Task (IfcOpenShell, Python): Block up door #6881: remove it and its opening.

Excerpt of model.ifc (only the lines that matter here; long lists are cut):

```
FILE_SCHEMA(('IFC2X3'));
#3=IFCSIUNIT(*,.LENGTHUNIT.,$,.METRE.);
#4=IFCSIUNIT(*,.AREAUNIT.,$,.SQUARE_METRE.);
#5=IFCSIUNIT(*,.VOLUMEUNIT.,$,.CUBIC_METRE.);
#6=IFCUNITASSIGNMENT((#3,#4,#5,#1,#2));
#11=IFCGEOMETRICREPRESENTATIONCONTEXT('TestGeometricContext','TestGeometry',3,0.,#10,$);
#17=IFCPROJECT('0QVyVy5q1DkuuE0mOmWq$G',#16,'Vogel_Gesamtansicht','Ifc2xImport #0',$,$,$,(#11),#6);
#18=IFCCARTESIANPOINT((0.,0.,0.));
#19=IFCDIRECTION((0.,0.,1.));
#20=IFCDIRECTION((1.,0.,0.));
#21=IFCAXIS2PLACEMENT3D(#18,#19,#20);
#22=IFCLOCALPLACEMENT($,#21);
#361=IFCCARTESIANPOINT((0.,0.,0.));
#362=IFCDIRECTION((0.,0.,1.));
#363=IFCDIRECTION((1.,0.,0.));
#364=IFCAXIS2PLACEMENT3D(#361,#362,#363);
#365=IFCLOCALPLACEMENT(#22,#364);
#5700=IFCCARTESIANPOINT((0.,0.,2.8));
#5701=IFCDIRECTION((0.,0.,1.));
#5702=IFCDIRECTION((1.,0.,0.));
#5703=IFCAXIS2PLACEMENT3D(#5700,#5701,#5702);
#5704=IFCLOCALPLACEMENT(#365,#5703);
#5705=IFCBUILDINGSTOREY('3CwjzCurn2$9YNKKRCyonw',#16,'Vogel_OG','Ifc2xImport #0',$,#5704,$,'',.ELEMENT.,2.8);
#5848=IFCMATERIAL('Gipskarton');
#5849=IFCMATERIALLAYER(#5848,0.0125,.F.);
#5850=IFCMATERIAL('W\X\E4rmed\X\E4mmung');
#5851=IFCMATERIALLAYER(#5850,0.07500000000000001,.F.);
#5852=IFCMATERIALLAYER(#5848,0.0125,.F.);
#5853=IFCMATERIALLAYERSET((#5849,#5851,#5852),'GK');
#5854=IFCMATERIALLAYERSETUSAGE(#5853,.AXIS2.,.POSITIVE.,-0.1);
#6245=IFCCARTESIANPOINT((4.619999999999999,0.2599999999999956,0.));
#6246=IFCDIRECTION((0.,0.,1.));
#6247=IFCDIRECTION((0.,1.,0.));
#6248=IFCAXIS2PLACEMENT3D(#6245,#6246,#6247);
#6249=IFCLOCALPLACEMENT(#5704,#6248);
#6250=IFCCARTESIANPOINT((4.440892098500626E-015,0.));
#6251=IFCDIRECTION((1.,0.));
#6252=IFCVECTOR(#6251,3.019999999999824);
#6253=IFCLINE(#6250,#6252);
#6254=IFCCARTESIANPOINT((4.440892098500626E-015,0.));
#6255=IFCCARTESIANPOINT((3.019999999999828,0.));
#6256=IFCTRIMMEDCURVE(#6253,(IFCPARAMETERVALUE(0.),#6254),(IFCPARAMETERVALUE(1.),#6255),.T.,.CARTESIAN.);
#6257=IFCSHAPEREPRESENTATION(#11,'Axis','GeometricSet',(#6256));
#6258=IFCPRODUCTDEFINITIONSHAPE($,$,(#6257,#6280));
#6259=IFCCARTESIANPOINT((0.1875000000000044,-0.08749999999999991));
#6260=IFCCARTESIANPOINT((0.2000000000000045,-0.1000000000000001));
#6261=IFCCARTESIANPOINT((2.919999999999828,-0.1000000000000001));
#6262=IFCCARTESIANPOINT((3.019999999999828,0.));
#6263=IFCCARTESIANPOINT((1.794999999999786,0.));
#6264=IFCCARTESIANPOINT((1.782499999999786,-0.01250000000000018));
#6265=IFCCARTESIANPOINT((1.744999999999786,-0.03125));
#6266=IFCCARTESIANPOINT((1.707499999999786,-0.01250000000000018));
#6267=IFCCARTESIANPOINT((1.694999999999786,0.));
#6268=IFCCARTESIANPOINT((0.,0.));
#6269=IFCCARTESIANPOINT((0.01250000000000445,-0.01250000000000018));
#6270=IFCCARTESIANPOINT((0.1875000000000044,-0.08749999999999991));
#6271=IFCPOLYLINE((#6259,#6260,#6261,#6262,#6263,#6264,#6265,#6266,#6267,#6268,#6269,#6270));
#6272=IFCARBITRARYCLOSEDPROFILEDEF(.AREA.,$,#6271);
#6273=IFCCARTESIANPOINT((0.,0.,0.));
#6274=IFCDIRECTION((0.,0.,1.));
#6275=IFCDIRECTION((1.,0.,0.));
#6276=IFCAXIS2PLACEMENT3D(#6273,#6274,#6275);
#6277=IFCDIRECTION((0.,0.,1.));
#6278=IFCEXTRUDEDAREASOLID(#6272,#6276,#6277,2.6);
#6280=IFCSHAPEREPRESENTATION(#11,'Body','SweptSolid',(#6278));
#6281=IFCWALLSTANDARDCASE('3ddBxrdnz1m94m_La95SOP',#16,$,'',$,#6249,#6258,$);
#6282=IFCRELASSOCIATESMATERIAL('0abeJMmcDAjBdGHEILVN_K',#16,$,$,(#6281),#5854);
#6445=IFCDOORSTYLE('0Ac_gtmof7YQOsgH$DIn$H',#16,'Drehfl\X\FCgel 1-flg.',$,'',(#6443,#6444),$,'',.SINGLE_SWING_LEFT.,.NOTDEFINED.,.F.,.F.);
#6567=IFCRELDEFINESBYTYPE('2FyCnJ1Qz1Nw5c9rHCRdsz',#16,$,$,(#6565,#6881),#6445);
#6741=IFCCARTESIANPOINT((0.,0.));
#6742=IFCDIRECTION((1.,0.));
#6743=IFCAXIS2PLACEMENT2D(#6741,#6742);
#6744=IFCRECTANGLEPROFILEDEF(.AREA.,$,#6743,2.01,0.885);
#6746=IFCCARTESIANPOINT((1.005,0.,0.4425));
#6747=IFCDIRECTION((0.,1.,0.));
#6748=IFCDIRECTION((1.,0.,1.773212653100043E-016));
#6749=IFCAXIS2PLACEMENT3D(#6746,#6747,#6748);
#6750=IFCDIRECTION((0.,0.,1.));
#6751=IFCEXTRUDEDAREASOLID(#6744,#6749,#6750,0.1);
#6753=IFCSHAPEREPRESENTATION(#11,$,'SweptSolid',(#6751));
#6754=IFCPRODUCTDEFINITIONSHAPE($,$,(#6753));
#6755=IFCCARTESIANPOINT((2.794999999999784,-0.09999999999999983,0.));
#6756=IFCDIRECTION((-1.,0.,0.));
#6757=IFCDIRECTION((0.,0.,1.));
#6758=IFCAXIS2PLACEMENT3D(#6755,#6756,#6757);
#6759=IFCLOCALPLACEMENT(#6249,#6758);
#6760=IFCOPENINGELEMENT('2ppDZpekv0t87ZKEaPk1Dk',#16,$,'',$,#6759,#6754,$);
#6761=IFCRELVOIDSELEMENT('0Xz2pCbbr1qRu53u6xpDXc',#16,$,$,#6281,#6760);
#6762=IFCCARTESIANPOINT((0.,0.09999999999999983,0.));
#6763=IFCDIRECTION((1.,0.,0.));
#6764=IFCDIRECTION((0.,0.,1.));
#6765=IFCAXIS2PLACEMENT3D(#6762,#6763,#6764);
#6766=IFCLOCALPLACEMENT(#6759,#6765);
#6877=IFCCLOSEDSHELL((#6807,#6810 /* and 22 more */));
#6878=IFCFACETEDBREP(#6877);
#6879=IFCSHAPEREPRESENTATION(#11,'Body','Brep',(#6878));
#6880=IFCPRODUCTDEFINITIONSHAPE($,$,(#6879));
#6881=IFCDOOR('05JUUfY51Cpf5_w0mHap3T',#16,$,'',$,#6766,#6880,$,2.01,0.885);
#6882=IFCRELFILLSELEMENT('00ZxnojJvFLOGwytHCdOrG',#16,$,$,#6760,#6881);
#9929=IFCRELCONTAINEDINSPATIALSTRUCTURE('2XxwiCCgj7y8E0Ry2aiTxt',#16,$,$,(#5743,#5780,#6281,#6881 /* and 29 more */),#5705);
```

```python
import ifcopenshell
import ifcopenshell.api.feature
import ifcopenshell.api.root
import ifcopenshell.geom
import ifcopenshell.util.shape

model = ifcopenshell.open("model.ifc")
settings = ifcopenshell.geom.settings()


def volume(element):
    """Net volume in cubic metres, openings subtracted."""
    shape = ifcopenshell.geom.create_shape(settings, element)
    return ifcopenshell.util.shape.get_volume(shape.geometry)


door = model.by_guid("05JUUfY51Cpf5_w0mHap3T")
opening = door.FillsVoids[0].RelatingOpeningElement
wall = opening.VoidsElements[0].RelatingBuildingElement
before = volume(wall)

ifcopenshell.api.root.remove_product(model, product=door)
ifcopenshell.api.feature.remove_feature(model, feature=opening)

after = volume(wall)

print(f"wall volume {before:.3f} -> {after:.3f} m3")

model.write("model_updated.ifc")
```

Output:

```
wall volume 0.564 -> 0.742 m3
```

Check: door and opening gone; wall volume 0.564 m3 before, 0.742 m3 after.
